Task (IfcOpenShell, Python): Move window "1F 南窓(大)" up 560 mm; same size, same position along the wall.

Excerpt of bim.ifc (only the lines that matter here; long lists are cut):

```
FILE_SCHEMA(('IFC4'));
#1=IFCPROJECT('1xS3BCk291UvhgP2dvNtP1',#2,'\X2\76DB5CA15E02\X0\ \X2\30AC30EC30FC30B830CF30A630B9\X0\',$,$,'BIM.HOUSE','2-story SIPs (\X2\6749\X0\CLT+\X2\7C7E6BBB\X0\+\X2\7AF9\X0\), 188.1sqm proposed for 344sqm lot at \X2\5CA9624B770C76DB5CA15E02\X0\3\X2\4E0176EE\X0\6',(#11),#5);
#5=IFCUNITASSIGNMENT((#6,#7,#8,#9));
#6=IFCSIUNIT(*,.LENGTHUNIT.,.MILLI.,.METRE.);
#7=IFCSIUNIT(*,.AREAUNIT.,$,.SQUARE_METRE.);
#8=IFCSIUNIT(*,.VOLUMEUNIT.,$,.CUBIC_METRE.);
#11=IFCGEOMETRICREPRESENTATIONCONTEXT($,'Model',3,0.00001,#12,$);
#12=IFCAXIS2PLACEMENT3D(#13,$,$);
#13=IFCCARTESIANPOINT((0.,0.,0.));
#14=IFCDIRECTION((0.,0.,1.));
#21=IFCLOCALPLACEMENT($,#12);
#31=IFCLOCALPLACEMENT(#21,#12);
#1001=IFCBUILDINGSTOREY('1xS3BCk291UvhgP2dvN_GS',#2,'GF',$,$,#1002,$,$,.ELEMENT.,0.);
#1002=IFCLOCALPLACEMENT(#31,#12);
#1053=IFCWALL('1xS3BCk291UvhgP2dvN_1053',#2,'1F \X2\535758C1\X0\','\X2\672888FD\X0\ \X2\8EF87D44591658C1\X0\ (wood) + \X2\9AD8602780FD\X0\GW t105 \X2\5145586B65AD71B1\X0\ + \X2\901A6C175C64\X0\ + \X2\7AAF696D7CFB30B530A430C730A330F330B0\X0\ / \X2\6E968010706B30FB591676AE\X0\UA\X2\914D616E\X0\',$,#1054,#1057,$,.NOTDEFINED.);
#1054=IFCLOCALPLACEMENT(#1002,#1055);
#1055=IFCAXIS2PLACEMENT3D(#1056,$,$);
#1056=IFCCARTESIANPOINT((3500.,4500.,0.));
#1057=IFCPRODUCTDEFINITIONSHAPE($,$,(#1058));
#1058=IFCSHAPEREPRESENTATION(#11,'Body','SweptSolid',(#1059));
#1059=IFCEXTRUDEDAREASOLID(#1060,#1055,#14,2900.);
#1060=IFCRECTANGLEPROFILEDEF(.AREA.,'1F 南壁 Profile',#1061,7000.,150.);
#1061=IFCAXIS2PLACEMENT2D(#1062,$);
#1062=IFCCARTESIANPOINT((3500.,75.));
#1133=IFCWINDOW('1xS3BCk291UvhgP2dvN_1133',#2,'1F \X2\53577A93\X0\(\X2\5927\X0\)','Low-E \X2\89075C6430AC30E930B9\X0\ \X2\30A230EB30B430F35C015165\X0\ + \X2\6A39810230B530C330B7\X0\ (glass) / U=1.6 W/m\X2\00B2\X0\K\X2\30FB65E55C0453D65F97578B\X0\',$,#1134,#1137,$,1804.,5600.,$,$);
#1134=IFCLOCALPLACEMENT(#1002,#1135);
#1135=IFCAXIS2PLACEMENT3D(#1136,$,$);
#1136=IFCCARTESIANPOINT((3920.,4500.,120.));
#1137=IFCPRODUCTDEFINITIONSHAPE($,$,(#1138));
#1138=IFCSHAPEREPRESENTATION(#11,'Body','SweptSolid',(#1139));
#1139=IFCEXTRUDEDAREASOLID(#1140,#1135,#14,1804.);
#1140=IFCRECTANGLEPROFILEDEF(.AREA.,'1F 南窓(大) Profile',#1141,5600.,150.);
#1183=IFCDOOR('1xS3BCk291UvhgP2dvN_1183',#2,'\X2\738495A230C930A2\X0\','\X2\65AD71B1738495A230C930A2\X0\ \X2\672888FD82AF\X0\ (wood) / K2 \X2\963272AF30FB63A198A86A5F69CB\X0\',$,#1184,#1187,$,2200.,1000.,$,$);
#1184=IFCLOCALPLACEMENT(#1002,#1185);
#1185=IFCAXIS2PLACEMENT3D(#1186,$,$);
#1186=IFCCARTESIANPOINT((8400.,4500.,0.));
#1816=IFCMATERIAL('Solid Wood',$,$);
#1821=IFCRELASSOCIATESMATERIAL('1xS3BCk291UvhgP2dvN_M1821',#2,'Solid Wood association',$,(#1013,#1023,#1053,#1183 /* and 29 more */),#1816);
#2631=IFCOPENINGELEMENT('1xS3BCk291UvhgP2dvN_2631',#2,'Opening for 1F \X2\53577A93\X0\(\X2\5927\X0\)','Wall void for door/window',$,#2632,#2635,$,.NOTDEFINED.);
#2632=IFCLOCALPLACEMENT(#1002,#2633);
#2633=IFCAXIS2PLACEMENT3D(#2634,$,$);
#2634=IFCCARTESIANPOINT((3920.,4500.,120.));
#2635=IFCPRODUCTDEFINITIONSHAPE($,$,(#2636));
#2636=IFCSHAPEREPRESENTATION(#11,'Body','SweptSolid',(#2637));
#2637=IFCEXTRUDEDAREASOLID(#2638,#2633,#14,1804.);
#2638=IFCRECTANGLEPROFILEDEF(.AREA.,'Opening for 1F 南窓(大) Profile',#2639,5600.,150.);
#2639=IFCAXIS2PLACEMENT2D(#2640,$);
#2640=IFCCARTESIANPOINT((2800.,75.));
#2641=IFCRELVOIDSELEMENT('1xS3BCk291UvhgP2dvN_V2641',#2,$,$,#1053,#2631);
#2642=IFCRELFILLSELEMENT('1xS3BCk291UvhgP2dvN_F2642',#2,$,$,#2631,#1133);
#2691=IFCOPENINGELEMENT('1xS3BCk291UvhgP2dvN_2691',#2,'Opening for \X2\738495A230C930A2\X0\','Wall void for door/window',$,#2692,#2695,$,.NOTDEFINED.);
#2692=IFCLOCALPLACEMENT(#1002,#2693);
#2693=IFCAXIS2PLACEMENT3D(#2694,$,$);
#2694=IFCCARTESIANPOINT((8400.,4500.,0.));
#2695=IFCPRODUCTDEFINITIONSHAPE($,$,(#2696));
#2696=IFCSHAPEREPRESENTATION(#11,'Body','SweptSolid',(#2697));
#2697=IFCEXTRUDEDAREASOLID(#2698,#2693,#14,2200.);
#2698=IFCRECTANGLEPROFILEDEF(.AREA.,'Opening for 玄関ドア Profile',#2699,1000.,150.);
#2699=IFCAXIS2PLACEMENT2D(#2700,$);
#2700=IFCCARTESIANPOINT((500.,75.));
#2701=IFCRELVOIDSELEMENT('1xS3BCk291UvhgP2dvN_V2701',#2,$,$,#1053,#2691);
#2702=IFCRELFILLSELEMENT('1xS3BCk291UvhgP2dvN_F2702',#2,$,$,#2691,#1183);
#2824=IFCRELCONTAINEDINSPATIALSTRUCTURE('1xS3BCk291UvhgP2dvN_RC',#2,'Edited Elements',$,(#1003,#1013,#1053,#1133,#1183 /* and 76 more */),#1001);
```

```python
import numpy as np
import ifcopenshell
import ifcopenshell.api.geometry
import ifcopenshell.util.placement
import ifcopenshell.util.unit

model = ifcopenshell.open("bim.ifc")
unit_scale = ifcopenshell.util.unit.calculate_unit_scale(model)

window = model.by_guid("1xS3BCk291UvhgP2dvN_1133")
opening = window.FillsVoids[0].RelatingOpeningElement
dz = 0.56 / unit_scale

shift = np.array([0.0, 0.0, dz])
# The window is not placed relative to its opening, so move both.
for product in (opening, window):
    matrix = ifcopenshell.util.placement.get_local_placement(product.ObjectPlacement)
    matrix[:3, 3] += shift
    ifcopenshell.api.geometry.edit_object_placement(model, product=product, matrix=matrix, is_si=False)

print(f"moved by {dz * unit_scale:+.3f} m")

model.write("bim-out.ifc")
```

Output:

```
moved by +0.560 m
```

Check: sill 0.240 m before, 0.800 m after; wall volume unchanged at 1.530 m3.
